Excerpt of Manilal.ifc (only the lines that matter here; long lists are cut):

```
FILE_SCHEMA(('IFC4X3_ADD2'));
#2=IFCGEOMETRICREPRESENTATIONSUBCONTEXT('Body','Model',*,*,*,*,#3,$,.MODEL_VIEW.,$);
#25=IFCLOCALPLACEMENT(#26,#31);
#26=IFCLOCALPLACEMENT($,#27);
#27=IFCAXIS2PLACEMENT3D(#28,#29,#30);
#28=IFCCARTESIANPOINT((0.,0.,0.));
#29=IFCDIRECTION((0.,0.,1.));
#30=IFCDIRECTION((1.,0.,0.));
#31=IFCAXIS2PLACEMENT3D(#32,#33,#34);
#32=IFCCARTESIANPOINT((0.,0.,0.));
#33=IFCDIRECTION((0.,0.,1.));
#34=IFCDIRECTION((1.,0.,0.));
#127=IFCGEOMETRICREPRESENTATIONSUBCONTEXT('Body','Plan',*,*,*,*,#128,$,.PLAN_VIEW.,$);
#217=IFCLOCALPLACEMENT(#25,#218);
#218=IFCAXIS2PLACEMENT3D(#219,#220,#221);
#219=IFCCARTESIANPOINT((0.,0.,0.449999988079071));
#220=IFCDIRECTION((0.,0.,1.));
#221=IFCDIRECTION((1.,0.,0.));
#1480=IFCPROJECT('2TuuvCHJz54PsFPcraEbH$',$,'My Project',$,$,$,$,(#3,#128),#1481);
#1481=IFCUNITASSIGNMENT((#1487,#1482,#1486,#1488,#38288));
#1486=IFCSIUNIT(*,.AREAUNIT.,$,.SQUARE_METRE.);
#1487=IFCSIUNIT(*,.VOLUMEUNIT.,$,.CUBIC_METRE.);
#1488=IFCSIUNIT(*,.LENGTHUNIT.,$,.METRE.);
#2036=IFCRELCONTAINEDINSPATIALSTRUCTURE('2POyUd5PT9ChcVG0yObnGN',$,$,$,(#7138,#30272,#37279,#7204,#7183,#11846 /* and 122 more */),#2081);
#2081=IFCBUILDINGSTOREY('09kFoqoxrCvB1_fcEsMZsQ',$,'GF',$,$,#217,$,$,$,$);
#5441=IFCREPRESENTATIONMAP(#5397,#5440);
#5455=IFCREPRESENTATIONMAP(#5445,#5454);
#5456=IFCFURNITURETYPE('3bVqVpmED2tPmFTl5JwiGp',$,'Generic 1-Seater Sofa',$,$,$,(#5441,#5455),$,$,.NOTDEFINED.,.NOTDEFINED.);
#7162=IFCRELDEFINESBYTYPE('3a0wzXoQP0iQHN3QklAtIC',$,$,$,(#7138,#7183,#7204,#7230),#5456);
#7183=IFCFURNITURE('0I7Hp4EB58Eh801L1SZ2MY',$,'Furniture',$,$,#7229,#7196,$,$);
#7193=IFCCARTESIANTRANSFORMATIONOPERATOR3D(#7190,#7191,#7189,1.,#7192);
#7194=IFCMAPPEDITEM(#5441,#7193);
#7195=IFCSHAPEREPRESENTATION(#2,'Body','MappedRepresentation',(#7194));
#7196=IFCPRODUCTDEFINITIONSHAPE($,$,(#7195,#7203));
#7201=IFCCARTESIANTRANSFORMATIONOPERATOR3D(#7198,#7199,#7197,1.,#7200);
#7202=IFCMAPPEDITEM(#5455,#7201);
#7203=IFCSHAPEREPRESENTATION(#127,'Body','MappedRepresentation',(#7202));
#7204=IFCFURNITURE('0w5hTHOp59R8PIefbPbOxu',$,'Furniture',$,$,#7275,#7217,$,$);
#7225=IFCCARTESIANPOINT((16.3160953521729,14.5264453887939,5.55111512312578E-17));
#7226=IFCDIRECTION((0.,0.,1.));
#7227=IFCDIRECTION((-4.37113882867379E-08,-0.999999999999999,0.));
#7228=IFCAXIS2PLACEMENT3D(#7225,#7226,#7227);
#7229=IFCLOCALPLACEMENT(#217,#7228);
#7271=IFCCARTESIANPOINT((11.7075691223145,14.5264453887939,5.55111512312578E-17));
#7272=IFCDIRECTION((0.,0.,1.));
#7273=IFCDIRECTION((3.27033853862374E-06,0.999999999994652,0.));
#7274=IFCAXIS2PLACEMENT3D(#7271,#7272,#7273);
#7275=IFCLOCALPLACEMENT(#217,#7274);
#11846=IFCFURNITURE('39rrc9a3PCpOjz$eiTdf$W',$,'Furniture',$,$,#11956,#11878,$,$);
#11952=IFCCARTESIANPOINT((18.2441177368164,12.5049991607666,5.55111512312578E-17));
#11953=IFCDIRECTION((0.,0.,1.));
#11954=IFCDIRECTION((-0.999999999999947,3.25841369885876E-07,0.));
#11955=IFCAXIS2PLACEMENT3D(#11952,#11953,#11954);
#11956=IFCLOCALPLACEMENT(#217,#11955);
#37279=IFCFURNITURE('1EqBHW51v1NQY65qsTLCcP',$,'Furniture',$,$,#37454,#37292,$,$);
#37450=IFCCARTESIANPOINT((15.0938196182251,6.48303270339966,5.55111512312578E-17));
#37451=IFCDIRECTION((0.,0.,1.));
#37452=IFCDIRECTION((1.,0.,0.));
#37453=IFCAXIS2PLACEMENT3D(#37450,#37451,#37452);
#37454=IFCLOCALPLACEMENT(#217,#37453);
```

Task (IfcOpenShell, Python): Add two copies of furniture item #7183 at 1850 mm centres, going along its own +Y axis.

```python
import ifcopenshell
import ifcopenshell.api.geometry
import ifcopenshell.api.root
import ifcopenshell.util.element
import ifcopenshell.util.placement

model = ifcopenshell.open("Manilal.ifc")

source = model.by_guid("0I7Hp4EB58Eh801L1SZ2MY")
base = ifcopenshell.util.placement.get_local_placement(source.ObjectPlacement)
step = base[:3, 1] * 1.85

for i in range(1, 3):
    copy = ifcopenshell.api.root.copy_class(model, product=source)
    copy.Representation = ifcopenshell.util.element.copy_deep(
        model, source.Representation, exclude=["IfcGeometricRepresentationContext", "IfcRepresentationMap"]
    )
    matrix = base.copy()
    matrix[:3, 3] += i * step
    print("added at", matrix[:3, 3].round(3) + 0.0)
    ifcopenshell.api.geometry.edit_object_placement(model, product=copy, matrix=matrix, is_si=False)

model.write("Manilal_rev.ifc")
```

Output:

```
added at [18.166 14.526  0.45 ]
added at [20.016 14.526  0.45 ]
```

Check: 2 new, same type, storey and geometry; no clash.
